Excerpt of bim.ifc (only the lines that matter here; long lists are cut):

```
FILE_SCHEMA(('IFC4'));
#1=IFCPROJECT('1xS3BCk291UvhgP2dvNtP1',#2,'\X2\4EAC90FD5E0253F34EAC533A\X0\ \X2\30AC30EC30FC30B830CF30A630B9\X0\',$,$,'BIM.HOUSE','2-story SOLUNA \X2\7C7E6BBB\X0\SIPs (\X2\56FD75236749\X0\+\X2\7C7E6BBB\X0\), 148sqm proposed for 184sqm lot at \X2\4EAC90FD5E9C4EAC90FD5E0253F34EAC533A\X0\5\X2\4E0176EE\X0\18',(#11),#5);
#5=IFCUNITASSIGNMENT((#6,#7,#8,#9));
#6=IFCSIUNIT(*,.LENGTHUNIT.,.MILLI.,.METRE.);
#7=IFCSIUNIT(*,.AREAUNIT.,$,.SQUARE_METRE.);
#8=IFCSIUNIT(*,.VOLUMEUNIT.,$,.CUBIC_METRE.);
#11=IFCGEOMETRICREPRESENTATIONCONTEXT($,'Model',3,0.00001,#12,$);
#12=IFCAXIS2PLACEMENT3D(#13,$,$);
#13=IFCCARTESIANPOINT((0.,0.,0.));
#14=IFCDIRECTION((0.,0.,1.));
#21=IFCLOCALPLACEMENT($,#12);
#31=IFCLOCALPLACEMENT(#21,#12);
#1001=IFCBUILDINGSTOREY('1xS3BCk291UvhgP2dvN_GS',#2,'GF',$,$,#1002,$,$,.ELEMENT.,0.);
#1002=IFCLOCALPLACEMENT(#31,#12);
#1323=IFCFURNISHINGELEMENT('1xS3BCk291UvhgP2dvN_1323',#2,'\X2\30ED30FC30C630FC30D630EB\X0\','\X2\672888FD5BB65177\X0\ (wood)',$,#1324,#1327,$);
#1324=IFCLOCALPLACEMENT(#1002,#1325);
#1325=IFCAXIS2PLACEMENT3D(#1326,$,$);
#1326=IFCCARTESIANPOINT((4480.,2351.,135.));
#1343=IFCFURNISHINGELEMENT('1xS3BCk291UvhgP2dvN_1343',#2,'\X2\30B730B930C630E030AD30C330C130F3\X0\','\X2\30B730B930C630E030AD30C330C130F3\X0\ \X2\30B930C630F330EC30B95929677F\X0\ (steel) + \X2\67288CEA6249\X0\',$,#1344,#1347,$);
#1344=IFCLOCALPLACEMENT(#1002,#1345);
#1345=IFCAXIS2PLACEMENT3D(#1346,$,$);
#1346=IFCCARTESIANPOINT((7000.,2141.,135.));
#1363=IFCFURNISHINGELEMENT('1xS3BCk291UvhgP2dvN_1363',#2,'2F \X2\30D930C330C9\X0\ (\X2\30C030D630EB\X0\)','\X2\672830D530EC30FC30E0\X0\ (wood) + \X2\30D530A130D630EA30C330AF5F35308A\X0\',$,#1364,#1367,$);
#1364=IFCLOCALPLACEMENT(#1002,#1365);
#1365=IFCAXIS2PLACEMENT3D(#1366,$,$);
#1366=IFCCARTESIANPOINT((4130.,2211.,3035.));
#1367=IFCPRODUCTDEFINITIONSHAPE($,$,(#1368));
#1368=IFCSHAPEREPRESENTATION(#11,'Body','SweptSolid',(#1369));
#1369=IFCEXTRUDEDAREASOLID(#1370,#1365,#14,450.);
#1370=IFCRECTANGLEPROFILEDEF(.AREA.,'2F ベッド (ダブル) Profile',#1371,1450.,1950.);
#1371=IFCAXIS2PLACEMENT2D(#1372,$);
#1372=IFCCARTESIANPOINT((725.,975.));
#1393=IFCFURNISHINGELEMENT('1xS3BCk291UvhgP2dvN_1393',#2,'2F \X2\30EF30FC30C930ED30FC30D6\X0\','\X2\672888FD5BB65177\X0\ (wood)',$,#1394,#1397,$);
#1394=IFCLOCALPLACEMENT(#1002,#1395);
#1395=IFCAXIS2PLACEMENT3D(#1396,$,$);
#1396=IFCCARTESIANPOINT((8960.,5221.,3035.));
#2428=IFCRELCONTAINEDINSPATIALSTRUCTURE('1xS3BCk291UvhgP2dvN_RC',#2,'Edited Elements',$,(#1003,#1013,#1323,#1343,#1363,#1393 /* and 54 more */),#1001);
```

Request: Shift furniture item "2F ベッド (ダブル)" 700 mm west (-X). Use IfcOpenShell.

```python
import ifcopenshell
import ifcopenshell.api.geometry
import ifcopenshell.util.placement
import ifcopenshell.util.unit

model = ifcopenshell.open("bim.ifc")
unit_scale = ifcopenshell.util.unit.calculate_unit_scale(model)

item = model.by_id(1363)
matrix = ifcopenshell.util.placement.get_local_placement(item.ObjectPlacement)
matrix[0, 3] -= 0.7 / unit_scale
ifcopenshell.api.geometry.edit_object_placement(model, product=item, matrix=matrix, is_si=False)

print(ifcopenshell.util.placement.get_local_placement(item.ObjectPlacement).round(3) + 0.0)

model.write("bim-out.ifc")
```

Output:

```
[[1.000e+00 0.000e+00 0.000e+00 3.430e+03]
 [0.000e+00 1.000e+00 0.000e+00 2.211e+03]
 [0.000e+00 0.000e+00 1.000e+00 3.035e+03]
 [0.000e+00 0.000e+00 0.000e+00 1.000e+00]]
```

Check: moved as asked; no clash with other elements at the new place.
